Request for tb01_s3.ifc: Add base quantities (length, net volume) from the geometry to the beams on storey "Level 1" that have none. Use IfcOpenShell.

First a look at what the model holds.

```python
import ifcopenshell
import ifcopenshell.util.element
import ifcopenshell.util.unit

model = ifcopenshell.open("tb01_s3.ifc")
print(model.schema)
for unit_type in ("LENGTHUNIT", "AREAUNIT", "VOLUMEUNIT"):
    print(unit_type, ifcopenshell.util.unit.calculate_unit_scale(model, unit_type))
storey = next(s for s in model.by_type("IfcBuildingStorey") if s.Name == "Level 1")
beams = [e for e in ifcopenshell.util.element.get_decomposition(storey) if e.is_a("IfcBeam")]
for e in sorted(beams, key=lambda e: e.id()):
    print(e.id(), e.is_a(), e.Name, list(ifcopenshell.util.element.get_psets(e, qtos_only=True)), sep=" | ")
```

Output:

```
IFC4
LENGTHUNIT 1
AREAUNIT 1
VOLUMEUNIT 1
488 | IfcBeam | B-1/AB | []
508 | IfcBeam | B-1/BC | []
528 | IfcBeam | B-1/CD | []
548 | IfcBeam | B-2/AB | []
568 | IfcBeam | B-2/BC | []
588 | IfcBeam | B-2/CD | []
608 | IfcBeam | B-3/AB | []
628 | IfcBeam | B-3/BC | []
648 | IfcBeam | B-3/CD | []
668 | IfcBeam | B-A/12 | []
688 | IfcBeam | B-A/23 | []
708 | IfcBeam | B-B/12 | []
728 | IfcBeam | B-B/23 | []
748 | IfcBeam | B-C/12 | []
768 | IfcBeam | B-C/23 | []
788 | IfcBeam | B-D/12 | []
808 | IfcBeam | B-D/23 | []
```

```python
import ifcopenshell
import ifcopenshell.api.pset
import ifcopenshell.geom
import ifcopenshell.util.element
import ifcopenshell.util.shape
import ifcopenshell.util.unit

model = ifcopenshell.open("tb01_s3.ifc")
unit_scale = ifcopenshell.util.unit.calculate_unit_scale(model)
volume_scale = ifcopenshell.util.unit.calculate_unit_scale(model, "VOLUMEUNIT")
settings = ifcopenshell.geom.settings()

storey = next(s for s in model.by_type("IfcBuildingStorey") if s.Name == "Level 1")
beams = [e for e in ifcopenshell.util.element.get_decomposition(storey) if e.is_a("IfcBeam")]

for e in sorted(beams, key=lambda e: e.id()):
    if ifcopenshell.util.element.get_psets(e, qtos_only=True, should_inherit=False):
        continue
    # Geometry comes back in metres, in the element's own axes.
    shape = ifcopenshell.geom.create_shape(settings, e)
    values = {
        "Length": ifcopenshell.util.shape.get_max_xyz(shape.geometry) / unit_scale,
        "NetVolume": ifcopenshell.util.shape.get_volume(shape.geometry) / volume_scale,
    }
    qto = ifcopenshell.api.pset.add_qto(model, product=e, name="Qto_BeamBaseQuantities")
    ifcopenshell.api.pset.edit_qto(model, qto=qto, properties=values)
    print(e.id(), {k: round(v, 3) for k, v in values.items()})

model.write("tb01_s3_rev.ifc")
```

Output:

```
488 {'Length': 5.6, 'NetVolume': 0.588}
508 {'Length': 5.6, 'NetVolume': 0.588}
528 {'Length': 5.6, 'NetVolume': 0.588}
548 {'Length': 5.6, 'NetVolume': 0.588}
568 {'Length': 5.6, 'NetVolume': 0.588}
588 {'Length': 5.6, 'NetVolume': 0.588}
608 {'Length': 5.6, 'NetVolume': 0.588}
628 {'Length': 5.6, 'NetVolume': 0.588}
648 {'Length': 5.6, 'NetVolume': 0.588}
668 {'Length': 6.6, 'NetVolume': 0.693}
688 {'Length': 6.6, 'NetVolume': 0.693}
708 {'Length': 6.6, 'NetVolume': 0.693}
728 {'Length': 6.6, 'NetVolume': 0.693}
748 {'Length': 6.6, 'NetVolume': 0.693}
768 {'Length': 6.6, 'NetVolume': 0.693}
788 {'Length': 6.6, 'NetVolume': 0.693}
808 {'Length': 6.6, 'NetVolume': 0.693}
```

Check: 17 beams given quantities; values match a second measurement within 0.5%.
